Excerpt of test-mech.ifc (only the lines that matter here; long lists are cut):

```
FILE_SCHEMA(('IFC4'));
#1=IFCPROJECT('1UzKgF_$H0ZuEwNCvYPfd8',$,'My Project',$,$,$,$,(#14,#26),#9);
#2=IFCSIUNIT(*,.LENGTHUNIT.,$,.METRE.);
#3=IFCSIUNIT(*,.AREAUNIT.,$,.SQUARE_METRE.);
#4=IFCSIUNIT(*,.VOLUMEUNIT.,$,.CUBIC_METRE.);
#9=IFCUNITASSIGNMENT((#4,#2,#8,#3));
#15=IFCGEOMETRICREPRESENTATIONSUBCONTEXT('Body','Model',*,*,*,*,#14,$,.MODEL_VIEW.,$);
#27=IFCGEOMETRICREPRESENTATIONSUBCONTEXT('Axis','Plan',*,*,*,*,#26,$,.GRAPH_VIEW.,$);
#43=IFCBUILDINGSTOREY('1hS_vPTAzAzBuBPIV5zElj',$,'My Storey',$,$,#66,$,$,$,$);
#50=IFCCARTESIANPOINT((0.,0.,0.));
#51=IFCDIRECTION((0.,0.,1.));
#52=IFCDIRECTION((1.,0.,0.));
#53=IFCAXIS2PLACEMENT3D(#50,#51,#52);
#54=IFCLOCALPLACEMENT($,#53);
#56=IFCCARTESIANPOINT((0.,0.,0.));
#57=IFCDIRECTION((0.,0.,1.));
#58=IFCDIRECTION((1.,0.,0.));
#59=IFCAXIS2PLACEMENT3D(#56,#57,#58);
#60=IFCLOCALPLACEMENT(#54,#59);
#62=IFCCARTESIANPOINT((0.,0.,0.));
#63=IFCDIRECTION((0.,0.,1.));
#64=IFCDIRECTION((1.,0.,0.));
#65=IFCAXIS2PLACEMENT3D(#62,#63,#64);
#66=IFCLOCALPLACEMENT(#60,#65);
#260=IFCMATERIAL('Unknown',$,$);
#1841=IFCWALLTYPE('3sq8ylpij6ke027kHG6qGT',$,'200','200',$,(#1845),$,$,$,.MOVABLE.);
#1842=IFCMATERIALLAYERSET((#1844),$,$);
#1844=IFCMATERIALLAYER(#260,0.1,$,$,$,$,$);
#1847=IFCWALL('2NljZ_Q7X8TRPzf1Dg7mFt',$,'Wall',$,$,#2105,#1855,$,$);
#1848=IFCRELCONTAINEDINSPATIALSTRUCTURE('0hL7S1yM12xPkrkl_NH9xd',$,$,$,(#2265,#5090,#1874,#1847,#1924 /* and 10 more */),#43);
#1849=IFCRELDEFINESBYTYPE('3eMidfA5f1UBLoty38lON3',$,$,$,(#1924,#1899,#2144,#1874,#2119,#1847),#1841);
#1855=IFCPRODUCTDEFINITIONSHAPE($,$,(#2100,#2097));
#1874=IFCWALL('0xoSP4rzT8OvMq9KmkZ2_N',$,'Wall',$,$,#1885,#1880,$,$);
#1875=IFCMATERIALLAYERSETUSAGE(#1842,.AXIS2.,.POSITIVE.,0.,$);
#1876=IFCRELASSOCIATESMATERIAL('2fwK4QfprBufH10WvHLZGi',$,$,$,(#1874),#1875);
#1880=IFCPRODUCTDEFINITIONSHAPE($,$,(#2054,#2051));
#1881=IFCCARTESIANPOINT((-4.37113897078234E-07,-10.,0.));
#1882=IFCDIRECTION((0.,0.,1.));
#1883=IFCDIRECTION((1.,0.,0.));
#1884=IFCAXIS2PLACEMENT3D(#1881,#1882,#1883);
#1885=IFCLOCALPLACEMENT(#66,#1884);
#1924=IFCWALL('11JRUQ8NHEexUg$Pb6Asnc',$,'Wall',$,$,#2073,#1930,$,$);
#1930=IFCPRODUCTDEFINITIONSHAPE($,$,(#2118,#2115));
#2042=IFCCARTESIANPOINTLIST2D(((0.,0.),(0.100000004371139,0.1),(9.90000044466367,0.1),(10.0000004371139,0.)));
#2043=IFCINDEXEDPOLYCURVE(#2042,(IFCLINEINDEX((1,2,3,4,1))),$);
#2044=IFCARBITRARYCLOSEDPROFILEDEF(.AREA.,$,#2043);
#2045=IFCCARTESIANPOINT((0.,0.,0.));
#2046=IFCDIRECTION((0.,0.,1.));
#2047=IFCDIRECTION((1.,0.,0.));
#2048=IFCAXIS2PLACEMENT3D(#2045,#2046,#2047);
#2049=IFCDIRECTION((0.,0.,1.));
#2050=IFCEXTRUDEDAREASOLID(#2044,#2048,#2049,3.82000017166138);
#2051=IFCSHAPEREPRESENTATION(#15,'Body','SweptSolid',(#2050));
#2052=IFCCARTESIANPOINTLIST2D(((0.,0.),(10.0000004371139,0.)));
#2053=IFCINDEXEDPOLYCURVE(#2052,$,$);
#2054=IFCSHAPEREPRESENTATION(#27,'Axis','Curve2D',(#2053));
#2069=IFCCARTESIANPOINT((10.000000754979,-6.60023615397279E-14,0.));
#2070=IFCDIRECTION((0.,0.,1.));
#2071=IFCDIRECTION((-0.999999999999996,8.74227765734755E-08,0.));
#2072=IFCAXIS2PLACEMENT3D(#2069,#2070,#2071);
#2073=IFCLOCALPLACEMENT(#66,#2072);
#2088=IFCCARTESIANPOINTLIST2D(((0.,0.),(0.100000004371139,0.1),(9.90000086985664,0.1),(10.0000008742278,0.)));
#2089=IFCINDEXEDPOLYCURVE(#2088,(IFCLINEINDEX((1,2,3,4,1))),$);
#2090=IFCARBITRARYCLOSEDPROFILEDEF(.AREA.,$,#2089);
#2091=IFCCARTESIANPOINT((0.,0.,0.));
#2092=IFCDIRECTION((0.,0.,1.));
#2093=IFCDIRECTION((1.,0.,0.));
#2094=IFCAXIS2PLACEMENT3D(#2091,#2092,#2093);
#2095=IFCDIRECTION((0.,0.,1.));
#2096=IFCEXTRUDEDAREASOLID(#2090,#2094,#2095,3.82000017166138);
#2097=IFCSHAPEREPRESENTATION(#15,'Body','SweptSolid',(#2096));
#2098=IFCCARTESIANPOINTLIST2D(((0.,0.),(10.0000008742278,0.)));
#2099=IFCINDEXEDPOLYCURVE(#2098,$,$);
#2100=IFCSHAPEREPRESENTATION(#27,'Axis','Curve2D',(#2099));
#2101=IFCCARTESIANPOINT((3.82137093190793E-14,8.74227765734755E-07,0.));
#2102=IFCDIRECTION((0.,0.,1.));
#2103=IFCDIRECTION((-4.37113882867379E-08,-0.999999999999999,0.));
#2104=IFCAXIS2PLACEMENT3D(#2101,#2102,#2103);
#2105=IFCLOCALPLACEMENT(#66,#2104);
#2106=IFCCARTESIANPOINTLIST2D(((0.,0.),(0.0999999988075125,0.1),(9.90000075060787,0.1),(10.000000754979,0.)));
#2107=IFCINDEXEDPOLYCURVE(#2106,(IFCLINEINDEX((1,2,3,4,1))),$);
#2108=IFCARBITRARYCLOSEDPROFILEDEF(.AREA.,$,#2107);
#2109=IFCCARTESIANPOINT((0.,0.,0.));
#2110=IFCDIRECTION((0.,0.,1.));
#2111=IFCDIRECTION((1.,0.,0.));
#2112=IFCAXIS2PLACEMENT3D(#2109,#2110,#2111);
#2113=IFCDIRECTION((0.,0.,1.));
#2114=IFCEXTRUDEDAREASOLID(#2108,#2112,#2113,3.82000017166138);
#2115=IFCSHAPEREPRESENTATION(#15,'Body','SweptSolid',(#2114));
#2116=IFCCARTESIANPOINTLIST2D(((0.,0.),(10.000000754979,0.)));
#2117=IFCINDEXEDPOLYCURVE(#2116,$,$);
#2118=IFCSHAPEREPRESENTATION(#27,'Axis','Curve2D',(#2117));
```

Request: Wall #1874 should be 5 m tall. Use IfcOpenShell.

```python
import ifcopenshell
import ifcopenshell.geom
import ifcopenshell.util.representation
import ifcopenshell.util.shape
import ifcopenshell.util.unit

model = ifcopenshell.open("test-mech.ifc")
unit_scale = ifcopenshell.util.unit.calculate_unit_scale(model)
settings = ifcopenshell.geom.settings()


def volume(element):
    """Net volume in cubic metres, openings subtracted."""
    shape = ifcopenshell.geom.create_shape(settings, element)
    return ifcopenshell.util.shape.get_volume(shape.geometry)


wall = model.by_id(1874)
before = volume(wall)

body = ifcopenshell.util.representation.get_representation(wall, "Model", "Body")
solid = body.Items[0]
old_height = solid.Depth
solid.Depth = 5 / unit_scale
after = volume(wall)

print(f"height {old_height:g} -> {solid.Depth:g}, volume {before:.3f} -> {after:.3f} m3")

model.write("test-mech-out.ifc")
```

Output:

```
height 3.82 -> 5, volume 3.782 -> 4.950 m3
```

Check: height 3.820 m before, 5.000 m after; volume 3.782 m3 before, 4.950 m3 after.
